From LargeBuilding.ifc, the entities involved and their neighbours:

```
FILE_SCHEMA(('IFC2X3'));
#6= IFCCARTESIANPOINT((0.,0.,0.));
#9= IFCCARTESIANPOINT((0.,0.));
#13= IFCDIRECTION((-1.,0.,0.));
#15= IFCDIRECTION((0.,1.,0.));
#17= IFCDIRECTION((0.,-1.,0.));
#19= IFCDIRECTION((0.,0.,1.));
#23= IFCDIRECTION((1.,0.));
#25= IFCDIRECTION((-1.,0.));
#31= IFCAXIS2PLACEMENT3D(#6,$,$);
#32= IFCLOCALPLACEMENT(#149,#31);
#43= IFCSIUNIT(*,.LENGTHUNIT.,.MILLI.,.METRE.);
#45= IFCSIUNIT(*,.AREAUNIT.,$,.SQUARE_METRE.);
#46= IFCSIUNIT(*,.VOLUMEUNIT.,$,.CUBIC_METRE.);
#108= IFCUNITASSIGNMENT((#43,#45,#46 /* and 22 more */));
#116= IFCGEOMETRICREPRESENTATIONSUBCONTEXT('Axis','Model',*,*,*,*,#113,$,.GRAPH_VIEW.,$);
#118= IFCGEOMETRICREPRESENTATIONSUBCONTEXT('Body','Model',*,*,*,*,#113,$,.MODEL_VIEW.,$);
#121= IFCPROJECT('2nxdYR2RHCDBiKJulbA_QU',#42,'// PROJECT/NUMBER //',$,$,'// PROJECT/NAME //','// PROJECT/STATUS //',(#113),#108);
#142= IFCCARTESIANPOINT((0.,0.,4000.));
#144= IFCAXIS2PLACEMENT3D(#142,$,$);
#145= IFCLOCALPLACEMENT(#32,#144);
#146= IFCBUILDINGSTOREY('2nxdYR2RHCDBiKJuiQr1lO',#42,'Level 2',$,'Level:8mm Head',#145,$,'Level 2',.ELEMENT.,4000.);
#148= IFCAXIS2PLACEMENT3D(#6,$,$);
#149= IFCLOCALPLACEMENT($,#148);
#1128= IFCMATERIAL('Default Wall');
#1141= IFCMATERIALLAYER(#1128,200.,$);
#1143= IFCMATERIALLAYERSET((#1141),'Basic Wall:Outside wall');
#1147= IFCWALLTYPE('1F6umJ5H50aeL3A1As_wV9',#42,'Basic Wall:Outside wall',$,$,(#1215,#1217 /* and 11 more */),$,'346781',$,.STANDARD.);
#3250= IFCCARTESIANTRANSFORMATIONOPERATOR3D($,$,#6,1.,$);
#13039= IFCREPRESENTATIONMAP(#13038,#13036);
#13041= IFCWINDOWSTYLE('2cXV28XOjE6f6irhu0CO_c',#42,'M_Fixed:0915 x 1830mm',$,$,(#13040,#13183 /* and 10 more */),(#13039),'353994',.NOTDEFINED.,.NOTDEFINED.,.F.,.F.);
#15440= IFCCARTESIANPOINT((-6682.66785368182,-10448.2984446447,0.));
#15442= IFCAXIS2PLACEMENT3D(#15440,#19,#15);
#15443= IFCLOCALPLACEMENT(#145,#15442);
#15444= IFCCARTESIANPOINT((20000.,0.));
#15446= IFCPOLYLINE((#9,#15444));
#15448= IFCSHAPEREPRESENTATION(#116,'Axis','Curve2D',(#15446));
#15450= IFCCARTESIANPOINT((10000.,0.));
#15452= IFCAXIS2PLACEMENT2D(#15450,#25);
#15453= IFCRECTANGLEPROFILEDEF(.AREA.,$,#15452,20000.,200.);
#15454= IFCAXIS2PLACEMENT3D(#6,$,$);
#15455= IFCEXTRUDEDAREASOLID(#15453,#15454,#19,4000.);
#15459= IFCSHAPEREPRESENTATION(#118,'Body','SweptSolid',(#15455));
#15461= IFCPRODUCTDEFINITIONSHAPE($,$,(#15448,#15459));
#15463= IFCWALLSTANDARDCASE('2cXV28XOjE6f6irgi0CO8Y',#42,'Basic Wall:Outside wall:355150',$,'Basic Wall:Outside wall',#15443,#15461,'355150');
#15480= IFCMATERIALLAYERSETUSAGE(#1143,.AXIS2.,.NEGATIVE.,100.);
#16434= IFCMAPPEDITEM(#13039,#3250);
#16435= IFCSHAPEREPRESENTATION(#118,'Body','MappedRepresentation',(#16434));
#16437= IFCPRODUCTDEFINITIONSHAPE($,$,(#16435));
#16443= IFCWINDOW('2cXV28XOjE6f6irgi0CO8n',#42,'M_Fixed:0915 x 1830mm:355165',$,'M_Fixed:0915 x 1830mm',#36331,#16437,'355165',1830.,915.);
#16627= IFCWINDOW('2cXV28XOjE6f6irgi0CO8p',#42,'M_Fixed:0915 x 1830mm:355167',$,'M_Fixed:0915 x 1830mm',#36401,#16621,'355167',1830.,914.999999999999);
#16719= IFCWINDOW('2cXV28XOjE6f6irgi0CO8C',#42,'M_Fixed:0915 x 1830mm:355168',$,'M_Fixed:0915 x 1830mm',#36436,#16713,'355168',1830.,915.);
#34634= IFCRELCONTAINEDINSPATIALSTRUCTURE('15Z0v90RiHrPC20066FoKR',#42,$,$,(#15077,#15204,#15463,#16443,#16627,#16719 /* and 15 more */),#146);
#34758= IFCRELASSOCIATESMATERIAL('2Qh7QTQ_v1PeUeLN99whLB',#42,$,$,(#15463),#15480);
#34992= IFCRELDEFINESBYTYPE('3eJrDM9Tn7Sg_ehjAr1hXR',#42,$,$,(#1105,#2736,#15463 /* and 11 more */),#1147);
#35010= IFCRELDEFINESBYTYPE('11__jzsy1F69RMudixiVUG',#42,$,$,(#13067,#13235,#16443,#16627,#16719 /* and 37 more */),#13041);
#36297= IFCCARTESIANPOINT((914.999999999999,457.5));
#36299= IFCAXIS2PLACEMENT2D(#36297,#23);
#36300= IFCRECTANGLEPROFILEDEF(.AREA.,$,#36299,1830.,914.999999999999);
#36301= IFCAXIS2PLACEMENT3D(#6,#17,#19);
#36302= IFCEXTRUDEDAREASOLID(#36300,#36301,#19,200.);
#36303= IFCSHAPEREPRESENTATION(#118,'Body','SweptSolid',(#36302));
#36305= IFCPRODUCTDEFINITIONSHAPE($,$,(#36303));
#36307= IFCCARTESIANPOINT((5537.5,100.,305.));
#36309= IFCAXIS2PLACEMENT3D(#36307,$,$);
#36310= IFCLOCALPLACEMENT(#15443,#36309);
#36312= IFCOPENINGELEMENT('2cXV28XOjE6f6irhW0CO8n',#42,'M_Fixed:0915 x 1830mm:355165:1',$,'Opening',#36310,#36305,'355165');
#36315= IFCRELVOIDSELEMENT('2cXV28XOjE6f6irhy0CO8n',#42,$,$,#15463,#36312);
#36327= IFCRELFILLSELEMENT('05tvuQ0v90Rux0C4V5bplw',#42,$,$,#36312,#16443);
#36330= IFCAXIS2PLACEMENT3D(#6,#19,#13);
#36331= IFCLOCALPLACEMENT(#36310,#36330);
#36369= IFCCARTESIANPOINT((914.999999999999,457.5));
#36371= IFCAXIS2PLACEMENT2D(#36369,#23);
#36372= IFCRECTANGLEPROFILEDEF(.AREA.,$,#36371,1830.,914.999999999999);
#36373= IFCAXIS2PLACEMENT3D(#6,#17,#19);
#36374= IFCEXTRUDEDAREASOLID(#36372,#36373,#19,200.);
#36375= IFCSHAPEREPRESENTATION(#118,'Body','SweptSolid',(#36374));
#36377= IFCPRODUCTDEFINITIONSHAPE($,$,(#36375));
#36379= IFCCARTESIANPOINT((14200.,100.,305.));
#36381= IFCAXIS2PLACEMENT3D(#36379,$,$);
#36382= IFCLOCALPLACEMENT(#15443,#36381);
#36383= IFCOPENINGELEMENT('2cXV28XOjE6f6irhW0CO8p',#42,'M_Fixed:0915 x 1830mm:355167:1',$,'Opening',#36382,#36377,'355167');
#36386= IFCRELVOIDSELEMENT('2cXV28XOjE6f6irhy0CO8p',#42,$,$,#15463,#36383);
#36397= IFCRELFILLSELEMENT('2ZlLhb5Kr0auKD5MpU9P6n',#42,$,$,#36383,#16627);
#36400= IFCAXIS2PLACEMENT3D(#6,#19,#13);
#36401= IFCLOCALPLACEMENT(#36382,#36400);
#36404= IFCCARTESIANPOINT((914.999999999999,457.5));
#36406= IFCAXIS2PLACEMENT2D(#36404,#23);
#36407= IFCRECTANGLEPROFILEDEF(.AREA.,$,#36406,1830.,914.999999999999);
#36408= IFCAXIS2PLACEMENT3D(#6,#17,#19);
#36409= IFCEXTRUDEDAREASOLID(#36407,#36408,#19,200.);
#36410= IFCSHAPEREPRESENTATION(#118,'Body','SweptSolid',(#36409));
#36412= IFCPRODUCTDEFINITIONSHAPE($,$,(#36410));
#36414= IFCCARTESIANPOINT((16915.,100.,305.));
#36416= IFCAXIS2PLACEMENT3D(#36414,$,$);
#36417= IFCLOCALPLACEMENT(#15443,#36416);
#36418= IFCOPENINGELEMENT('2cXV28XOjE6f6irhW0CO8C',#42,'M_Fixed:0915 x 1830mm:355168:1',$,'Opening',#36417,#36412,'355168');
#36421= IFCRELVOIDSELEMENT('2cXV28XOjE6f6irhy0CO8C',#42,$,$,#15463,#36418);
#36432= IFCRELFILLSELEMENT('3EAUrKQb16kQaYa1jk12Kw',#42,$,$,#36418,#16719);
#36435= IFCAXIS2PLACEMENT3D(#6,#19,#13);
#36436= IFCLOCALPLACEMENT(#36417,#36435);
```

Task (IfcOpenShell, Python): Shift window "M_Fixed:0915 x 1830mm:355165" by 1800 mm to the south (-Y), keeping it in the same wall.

```python
import ifcopenshell
import ifcopenshell.api.geometry
import ifcopenshell.util.placement

model = ifcopenshell.open("LargeBuilding.ifc")

window = model.by_id(16443)
opening = window.FillsVoids[0].RelatingOpeningElement
wall = opening.VoidsElements[0].RelatingBuildingElement

wall_matrix = ifcopenshell.util.placement.get_local_placement(wall.ObjectPlacement)
shift = wall_matrix[:3, 0] * -1800.0
before = ifcopenshell.util.placement.get_local_placement(window.ObjectPlacement)[:3, 3].copy()

# The window is placed relative to its opening, so it follows when the opening moves.
matrix = ifcopenshell.util.placement.get_local_placement(opening.ObjectPlacement)
matrix[:3, 3] += shift
ifcopenshell.api.geometry.edit_object_placement(
    model, product=opening, matrix=matrix, is_si=False, should_transform_children=True
)

after = ifcopenshell.util.placement.get_local_placement(window.ObjectPlacement)[:3, 3]
print("window moved by", (after - before).round(3) + 0.0)

model.write("LargeBuilding_updated.ifc")
```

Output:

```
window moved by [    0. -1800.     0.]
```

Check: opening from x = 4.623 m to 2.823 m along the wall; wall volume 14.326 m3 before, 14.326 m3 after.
